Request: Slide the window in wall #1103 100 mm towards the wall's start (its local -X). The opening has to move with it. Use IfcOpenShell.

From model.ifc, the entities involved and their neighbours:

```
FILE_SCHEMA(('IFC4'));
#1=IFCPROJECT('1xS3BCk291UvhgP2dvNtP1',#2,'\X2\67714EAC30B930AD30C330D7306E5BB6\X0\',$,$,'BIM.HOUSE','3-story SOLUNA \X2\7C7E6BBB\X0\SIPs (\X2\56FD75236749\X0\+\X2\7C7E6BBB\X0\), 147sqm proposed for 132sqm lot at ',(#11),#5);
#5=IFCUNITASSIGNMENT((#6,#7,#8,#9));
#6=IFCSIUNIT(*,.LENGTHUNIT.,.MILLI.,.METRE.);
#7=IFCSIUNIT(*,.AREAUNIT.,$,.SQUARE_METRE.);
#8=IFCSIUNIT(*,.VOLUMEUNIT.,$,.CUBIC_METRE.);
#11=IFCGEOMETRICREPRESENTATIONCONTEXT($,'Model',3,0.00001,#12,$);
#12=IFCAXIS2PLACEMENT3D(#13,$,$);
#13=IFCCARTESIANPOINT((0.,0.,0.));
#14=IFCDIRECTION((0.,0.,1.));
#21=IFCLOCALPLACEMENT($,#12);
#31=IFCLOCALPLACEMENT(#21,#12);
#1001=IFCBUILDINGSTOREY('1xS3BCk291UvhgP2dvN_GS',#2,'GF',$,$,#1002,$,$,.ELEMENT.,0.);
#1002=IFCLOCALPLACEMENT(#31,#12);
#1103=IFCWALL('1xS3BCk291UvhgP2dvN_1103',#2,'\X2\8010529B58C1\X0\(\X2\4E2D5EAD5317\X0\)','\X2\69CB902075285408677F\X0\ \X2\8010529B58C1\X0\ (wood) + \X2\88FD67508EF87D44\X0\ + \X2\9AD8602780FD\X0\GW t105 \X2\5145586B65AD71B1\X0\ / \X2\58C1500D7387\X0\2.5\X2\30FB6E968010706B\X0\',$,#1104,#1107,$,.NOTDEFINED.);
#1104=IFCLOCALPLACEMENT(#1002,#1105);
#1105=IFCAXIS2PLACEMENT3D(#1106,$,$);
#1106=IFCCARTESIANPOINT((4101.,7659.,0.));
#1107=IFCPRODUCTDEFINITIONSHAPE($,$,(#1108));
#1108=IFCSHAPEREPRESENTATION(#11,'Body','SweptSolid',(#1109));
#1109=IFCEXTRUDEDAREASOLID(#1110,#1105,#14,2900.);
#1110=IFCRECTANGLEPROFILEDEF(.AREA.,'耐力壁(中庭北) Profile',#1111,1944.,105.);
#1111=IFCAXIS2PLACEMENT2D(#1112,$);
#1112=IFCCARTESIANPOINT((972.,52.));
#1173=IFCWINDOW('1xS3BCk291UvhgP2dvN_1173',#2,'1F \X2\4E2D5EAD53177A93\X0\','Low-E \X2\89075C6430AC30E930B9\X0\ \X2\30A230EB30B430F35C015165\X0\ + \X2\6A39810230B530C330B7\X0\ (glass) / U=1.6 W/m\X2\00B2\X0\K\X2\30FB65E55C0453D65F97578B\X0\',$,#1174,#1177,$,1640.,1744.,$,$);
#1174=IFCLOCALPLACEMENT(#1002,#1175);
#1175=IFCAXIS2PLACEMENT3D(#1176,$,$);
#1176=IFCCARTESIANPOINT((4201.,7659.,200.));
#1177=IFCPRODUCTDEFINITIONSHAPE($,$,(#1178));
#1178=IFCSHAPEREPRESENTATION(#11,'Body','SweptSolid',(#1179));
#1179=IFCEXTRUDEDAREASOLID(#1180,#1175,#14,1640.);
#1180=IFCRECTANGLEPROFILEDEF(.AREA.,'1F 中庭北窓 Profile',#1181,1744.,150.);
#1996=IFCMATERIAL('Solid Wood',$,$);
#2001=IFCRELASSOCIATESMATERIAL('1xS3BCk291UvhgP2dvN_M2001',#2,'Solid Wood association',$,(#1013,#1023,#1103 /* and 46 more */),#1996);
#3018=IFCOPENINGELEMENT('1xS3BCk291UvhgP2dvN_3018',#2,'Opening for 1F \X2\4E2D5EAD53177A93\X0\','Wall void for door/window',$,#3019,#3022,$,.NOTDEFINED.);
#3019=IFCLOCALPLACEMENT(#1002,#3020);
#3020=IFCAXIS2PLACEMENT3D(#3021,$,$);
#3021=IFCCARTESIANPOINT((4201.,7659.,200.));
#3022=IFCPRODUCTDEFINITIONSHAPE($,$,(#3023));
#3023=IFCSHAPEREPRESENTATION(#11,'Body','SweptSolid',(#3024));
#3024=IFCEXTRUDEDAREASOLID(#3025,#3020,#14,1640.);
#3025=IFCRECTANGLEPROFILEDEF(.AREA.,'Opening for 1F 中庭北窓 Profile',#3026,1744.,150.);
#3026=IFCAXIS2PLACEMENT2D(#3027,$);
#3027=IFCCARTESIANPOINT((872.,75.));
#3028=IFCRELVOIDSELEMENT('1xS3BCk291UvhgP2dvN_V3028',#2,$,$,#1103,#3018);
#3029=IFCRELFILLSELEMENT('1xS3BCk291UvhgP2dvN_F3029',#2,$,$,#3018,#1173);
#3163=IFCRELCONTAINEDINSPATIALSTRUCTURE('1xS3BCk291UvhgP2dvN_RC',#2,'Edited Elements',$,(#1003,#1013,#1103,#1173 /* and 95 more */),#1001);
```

```python
import ifcopenshell
import ifcopenshell.api.geometry
import ifcopenshell.util.placement
import ifcopenshell.util.unit

model = ifcopenshell.open("model.ifc")
unit_scale = ifcopenshell.util.unit.calculate_unit_scale(model)

window = model.by_guid("1xS3BCk291UvhgP2dvN_1173")
opening = window.FillsVoids[0].RelatingOpeningElement
wall = opening.VoidsElements[0].RelatingBuildingElement

wall_matrix = ifcopenshell.util.placement.get_local_placement(wall.ObjectPlacement)
shift = wall_matrix[:3, 0] * -0.1 / unit_scale
before = ifcopenshell.util.placement.get_local_placement(window.ObjectPlacement)[:3, 3].copy()

# The window is not placed relative to its opening, so move both.
for product in (opening, window):
    matrix = ifcopenshell.util.placement.get_local_placement(product.ObjectPlacement)
    matrix[:3, 3] += shift
    ifcopenshell.api.geometry.edit_object_placement(model, product=product, matrix=matrix, is_si=False)

after = ifcopenshell.util.placement.get_local_placement(window.ObjectPlacement)[:3, 3]
print("window moved by", (after - before).round(3) + 0.0)

model.write("model_rev.ifc")
```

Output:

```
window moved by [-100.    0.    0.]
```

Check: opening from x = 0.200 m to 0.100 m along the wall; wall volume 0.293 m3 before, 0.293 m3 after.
